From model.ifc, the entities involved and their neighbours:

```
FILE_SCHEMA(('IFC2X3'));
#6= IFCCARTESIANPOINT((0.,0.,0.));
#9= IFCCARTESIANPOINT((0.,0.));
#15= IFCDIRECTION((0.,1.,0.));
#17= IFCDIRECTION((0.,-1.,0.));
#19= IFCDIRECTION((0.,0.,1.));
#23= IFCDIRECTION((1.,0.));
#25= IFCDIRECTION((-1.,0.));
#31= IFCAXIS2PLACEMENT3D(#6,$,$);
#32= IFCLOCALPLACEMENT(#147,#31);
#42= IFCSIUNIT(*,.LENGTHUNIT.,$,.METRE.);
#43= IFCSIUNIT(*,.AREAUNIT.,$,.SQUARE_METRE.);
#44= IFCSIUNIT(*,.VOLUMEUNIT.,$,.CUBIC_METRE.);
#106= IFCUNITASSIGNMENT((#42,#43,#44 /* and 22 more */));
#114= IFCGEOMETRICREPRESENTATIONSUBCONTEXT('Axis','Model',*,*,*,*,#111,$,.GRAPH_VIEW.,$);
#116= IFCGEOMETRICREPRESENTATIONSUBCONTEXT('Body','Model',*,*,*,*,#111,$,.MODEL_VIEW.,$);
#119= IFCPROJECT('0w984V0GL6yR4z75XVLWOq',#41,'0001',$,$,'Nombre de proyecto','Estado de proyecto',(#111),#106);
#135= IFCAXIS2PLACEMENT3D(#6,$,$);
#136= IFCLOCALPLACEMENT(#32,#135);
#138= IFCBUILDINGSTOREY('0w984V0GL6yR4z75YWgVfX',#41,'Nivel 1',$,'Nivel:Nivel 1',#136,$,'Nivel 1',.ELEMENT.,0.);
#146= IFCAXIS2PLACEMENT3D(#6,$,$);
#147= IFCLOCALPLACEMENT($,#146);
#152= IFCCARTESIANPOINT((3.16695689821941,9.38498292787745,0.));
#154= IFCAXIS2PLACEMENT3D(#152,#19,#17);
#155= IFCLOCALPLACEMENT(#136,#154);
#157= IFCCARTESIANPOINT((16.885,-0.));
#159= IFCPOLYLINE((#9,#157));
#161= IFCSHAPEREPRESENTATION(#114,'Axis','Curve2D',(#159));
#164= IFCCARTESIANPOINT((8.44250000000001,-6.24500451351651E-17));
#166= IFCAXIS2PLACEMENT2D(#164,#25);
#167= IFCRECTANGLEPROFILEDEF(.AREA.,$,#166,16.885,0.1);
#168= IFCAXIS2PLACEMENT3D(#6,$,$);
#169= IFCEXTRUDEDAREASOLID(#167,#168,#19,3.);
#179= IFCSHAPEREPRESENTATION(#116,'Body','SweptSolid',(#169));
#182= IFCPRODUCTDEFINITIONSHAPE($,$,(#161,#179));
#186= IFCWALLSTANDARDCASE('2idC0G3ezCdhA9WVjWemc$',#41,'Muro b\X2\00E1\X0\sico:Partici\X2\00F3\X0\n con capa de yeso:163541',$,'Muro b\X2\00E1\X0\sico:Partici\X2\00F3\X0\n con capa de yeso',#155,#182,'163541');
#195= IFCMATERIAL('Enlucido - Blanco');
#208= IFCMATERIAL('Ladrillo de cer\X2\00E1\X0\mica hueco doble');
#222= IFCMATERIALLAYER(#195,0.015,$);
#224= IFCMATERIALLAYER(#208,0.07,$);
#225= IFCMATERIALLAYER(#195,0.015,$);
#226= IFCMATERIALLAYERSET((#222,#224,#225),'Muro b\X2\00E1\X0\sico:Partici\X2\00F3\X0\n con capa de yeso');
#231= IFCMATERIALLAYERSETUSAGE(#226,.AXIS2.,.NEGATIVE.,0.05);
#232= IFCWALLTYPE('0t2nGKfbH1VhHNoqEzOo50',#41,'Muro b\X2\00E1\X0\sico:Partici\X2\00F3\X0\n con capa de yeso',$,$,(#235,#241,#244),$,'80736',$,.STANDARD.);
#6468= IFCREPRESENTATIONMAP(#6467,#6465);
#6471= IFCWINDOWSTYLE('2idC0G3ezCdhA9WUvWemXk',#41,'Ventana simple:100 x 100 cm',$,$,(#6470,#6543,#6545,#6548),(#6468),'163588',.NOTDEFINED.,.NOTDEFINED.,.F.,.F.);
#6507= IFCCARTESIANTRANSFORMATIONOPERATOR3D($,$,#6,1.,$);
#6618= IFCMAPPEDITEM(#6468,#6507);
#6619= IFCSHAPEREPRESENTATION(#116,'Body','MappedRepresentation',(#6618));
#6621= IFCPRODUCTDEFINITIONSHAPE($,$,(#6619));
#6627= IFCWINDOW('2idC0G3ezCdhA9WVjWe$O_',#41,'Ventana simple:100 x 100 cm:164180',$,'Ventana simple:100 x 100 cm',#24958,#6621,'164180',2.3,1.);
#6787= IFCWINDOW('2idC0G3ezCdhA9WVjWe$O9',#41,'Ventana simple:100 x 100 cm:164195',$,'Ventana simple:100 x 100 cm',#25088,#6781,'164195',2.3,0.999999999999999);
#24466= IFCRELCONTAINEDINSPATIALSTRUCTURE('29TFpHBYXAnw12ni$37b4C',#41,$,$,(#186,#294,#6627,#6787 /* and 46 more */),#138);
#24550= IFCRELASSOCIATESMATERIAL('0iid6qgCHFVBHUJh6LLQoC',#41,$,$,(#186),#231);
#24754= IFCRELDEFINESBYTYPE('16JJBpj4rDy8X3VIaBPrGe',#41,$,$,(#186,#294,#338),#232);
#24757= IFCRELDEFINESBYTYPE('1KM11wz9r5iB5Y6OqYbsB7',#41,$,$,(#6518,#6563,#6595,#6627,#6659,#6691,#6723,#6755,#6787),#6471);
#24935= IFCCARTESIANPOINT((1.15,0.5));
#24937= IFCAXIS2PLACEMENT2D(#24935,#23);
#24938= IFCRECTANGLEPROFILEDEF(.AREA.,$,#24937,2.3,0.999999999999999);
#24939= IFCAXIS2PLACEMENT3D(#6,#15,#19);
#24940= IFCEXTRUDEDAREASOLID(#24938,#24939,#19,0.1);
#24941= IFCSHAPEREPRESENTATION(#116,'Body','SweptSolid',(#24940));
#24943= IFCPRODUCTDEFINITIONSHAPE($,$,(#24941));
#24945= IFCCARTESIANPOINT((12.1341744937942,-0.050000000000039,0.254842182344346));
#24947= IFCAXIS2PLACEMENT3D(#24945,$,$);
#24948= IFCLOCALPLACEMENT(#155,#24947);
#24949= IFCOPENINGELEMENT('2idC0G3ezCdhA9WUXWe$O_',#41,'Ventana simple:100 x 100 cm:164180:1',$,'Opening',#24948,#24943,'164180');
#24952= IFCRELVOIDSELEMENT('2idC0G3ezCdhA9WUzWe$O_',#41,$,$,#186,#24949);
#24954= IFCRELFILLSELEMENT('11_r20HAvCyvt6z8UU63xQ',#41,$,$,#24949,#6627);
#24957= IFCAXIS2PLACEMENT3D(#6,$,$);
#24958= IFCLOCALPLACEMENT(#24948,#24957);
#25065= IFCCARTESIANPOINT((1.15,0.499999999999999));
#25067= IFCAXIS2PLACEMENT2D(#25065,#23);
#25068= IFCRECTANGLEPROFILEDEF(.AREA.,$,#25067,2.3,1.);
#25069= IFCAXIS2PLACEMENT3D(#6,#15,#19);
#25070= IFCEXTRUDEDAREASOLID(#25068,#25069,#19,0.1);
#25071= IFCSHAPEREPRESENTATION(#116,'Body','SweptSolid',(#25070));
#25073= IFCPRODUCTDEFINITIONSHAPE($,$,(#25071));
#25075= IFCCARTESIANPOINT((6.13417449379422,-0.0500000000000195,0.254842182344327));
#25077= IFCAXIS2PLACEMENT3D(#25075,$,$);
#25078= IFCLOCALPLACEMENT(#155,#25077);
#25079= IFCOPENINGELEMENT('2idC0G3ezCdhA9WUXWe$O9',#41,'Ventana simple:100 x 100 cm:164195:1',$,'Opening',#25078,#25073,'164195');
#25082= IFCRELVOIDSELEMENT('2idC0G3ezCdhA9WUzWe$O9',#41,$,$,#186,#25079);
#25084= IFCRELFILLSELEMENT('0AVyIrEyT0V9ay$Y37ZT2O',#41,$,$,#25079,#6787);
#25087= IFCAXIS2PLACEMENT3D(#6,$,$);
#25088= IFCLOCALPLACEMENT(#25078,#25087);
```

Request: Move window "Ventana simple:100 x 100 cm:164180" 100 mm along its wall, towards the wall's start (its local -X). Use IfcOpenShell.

```python
import ifcopenshell
import ifcopenshell.api.geometry
import ifcopenshell.util.placement
import ifcopenshell.util.unit

model = ifcopenshell.open("model.ifc")
unit_scale = ifcopenshell.util.unit.calculate_unit_scale(model)

window = model.by_id(6627)
opening = window.FillsVoids[0].RelatingOpeningElement
wall = opening.VoidsElements[0].RelatingBuildingElement

wall_matrix = ifcopenshell.util.placement.get_local_placement(wall.ObjectPlacement)
shift = wall_matrix[:3, 0] * -0.1 / unit_scale
before = ifcopenshell.util.placement.get_local_placement(window.ObjectPlacement)[:3, 3].copy()

# The window is placed relative to its opening, so it follows when the opening moves.
matrix = ifcopenshell.util.placement.get_local_placement(opening.ObjectPlacement)
matrix[:3, 3] += shift
ifcopenshell.api.geometry.edit_object_placement(
    model, product=opening, matrix=matrix, is_si=False, should_transform_children=True
)

after = ifcopenshell.util.placement.get_local_placement(window.ObjectPlacement)[:3, 3]
print("window moved by", (after - before).round(3) + 0.0)

model.write("model_edited.ifc")
```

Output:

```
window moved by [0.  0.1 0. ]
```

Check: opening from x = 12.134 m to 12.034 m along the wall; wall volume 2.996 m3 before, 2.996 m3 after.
